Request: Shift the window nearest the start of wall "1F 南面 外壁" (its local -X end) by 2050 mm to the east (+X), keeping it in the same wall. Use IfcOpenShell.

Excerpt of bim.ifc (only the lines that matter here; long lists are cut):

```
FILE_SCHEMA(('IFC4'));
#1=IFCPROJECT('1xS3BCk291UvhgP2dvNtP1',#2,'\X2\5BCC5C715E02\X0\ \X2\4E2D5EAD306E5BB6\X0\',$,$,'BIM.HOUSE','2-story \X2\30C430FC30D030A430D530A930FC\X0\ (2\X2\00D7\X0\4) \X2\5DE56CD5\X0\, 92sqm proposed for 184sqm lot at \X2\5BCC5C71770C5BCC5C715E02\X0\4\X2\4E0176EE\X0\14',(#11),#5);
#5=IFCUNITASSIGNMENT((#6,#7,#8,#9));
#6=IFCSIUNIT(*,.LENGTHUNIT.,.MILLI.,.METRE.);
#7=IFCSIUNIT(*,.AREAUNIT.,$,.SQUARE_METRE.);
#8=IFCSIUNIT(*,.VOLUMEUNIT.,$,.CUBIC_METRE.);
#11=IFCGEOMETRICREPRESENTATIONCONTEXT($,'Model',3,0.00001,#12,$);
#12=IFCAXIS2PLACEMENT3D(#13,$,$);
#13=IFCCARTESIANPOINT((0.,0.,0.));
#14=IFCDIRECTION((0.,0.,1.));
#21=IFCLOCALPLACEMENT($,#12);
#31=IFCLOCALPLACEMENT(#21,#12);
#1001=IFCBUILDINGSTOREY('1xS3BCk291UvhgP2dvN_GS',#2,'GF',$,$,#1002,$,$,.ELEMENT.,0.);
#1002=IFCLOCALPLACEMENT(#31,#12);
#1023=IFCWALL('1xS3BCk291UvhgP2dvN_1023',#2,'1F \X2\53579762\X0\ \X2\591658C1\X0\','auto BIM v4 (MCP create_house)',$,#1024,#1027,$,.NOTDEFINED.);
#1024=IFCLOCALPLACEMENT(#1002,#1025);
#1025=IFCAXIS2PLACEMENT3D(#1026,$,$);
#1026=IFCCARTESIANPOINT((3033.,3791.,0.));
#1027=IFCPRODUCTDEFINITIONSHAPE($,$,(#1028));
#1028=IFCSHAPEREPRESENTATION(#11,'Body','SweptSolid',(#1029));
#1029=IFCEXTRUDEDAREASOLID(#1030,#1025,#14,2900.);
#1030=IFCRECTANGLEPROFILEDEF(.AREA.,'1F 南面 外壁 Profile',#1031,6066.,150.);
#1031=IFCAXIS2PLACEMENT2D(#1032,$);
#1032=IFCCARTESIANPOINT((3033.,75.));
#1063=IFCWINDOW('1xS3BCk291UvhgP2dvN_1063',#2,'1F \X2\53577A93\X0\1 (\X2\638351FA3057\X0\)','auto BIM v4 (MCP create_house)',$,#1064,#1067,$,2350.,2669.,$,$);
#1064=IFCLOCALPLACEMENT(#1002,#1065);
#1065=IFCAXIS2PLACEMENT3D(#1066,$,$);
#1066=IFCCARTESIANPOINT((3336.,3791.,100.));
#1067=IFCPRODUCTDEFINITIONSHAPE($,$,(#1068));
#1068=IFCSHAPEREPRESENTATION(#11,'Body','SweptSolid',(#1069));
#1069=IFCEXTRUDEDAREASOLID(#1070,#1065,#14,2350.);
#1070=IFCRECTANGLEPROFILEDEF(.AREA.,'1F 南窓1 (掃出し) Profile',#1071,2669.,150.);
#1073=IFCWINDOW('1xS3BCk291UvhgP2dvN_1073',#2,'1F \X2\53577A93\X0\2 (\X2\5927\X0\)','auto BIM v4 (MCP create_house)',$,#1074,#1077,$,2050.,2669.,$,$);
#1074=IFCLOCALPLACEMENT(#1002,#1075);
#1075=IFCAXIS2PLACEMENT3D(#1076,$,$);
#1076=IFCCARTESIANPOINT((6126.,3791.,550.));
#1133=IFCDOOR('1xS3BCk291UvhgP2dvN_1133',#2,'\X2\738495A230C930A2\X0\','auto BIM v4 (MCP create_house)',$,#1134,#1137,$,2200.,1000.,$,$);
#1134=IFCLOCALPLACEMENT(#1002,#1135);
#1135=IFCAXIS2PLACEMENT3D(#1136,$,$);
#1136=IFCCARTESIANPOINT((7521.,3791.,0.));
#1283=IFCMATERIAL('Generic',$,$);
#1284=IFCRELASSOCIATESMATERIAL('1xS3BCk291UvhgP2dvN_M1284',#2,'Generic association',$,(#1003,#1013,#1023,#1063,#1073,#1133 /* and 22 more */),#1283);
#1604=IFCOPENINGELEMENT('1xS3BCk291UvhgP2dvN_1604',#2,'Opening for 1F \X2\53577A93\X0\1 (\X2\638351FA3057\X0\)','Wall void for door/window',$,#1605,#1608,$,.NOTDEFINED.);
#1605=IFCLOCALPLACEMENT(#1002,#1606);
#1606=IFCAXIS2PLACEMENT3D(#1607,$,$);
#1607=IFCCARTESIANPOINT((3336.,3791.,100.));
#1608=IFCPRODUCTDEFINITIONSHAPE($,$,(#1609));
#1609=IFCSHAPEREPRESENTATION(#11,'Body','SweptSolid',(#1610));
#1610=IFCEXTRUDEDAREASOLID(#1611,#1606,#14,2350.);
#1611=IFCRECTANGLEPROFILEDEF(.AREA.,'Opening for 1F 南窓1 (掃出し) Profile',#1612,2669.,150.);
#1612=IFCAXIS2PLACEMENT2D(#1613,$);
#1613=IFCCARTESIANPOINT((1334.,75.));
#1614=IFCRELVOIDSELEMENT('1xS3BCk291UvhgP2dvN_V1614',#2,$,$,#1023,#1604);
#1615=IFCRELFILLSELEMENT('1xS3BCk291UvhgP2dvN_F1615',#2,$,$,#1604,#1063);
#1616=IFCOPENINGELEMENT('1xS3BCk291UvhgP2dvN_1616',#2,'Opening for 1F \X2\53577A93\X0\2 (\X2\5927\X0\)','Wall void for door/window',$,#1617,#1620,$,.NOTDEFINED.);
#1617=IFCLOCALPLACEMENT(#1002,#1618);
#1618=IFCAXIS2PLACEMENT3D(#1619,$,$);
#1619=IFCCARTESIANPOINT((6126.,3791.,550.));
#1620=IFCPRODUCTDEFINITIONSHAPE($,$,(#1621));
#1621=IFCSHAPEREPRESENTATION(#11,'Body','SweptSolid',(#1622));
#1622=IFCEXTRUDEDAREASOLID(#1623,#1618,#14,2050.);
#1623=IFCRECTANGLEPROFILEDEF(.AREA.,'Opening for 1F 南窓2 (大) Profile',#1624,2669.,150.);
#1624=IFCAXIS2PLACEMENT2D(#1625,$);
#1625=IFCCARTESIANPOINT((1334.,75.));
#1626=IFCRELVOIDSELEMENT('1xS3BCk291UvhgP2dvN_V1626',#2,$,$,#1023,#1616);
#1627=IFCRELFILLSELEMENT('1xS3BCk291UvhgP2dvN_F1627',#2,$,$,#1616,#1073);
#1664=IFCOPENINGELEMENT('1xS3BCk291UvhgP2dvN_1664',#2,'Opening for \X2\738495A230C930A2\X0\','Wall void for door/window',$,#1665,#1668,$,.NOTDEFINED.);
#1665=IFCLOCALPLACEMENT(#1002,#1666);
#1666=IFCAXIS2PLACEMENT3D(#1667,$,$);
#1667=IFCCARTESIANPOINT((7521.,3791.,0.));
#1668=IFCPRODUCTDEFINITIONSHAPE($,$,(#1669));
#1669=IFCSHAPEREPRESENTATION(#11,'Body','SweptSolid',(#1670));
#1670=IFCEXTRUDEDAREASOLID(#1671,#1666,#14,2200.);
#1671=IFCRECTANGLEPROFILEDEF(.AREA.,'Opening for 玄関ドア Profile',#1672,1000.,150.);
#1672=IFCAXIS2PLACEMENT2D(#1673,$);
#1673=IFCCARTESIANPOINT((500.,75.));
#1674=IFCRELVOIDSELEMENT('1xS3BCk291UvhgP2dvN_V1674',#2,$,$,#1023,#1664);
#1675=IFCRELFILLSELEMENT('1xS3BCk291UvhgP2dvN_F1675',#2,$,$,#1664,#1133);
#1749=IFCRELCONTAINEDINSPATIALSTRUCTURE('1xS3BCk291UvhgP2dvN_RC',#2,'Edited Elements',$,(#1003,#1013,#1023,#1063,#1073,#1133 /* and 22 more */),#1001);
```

```python
import ifcopenshell
import ifcopenshell.api.geometry
import ifcopenshell.util.placement
import ifcopenshell.util.unit

model = ifcopenshell.open("bim.ifc")
unit_scale = ifcopenshell.util.unit.calculate_unit_scale(model)

window = model.by_guid("1xS3BCk291UvhgP2dvN_1063")
opening = window.FillsVoids[0].RelatingOpeningElement
wall = opening.VoidsElements[0].RelatingBuildingElement

wall_matrix = ifcopenshell.util.placement.get_local_placement(wall.ObjectPlacement)
shift = wall_matrix[:3, 0] * 2.05 / unit_scale
before = ifcopenshell.util.placement.get_local_placement(window.ObjectPlacement)[:3, 3].copy()

# The window is not placed relative to its opening, so move both.
for product in (opening, window):
    matrix = ifcopenshell.util.placement.get_local_placement(product.ObjectPlacement)
    matrix[:3, 3] += shift
    ifcopenshell.api.geometry.edit_object_placement(model, product=product, matrix=matrix, is_si=False)

after = ifcopenshell.util.placement.get_local_placement(window.ObjectPlacement)[:3, 3]
print("window moved by", (after - before).round(3) + 0.0)

model.write("bim_v2.ifc")
```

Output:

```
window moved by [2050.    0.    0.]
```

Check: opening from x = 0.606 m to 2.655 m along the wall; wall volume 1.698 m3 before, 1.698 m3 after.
